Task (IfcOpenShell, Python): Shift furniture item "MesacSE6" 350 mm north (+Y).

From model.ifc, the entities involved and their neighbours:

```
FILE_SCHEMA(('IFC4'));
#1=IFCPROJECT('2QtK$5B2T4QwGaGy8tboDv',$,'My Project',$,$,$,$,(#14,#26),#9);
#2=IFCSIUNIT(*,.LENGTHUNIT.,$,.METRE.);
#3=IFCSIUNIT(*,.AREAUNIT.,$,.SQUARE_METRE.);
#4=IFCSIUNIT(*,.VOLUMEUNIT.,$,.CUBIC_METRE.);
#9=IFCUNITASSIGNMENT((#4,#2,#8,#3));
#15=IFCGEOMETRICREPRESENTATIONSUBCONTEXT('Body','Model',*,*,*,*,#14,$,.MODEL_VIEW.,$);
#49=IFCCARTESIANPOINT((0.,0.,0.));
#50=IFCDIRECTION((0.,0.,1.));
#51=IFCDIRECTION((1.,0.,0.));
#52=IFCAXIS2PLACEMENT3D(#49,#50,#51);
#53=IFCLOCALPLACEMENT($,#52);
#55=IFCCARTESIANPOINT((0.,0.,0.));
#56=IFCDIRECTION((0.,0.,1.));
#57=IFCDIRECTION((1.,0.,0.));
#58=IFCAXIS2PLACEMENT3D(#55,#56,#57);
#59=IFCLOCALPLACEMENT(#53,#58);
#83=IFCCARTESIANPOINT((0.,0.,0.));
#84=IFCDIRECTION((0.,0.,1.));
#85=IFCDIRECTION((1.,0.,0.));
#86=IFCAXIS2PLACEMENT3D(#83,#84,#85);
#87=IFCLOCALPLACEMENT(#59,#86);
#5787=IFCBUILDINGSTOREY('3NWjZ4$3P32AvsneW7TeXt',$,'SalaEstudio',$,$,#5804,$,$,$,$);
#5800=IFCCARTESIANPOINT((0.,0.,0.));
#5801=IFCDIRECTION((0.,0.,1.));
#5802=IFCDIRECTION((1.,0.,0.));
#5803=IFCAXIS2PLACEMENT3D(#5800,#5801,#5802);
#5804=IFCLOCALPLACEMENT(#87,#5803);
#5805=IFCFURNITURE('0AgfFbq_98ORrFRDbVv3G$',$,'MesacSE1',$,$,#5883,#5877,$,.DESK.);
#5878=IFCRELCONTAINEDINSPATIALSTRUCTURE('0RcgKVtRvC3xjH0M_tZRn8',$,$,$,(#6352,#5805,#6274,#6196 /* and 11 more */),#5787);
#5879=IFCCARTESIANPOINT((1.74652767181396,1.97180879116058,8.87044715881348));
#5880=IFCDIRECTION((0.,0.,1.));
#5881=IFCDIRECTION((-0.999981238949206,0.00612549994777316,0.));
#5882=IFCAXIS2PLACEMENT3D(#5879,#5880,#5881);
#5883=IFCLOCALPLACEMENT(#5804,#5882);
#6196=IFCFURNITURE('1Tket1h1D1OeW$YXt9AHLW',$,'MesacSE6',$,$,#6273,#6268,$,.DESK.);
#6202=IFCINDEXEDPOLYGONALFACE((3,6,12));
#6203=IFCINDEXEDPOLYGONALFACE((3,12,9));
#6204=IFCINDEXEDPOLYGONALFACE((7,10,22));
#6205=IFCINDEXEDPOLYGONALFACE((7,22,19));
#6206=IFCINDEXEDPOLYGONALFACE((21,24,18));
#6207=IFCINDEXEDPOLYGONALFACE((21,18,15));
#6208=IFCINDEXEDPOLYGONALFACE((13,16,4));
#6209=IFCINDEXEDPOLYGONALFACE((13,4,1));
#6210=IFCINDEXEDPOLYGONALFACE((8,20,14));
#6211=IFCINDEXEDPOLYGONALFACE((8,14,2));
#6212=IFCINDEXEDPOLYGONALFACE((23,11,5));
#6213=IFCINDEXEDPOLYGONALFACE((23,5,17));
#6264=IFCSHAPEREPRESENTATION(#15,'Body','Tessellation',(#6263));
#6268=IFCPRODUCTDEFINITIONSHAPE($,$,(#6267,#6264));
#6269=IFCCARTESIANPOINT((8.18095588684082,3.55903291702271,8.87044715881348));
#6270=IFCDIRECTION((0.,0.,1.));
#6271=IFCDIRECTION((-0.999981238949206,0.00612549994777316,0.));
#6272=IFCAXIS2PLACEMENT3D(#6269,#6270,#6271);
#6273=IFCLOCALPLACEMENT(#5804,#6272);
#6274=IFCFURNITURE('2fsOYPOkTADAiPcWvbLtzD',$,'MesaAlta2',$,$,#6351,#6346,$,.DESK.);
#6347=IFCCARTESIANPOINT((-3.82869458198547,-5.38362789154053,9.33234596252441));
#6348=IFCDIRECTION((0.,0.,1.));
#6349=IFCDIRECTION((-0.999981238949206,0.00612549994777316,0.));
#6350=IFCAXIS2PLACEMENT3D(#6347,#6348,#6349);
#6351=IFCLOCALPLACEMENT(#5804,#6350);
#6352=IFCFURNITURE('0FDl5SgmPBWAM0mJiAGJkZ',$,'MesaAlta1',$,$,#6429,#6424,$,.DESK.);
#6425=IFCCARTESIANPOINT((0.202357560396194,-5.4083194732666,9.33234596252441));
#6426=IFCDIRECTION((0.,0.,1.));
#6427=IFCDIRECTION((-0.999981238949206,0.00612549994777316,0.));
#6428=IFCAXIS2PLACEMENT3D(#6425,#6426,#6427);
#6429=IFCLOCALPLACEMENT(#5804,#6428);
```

```python
import ifcopenshell
import ifcopenshell.api.geometry
import ifcopenshell.util.placement
import ifcopenshell.util.unit

model = ifcopenshell.open("model.ifc")
unit_scale = ifcopenshell.util.unit.calculate_unit_scale(model)

item = model.by_guid("1Tket1h1D1OeW$YXt9AHLW")
matrix = ifcopenshell.util.placement.get_local_placement(item.ObjectPlacement)
matrix[1, 3] += 0.35 / unit_scale
ifcopenshell.api.geometry.edit_object_placement(model, product=item, matrix=matrix, is_si=False)

print(ifcopenshell.util.placement.get_local_placement(item.ObjectPlacement).round(3) + 0.0)

model.write("model_v2.ifc")
```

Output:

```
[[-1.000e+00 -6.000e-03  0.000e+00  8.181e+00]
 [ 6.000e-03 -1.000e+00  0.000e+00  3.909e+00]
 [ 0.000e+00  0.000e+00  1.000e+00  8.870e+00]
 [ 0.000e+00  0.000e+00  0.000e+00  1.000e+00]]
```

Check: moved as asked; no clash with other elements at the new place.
